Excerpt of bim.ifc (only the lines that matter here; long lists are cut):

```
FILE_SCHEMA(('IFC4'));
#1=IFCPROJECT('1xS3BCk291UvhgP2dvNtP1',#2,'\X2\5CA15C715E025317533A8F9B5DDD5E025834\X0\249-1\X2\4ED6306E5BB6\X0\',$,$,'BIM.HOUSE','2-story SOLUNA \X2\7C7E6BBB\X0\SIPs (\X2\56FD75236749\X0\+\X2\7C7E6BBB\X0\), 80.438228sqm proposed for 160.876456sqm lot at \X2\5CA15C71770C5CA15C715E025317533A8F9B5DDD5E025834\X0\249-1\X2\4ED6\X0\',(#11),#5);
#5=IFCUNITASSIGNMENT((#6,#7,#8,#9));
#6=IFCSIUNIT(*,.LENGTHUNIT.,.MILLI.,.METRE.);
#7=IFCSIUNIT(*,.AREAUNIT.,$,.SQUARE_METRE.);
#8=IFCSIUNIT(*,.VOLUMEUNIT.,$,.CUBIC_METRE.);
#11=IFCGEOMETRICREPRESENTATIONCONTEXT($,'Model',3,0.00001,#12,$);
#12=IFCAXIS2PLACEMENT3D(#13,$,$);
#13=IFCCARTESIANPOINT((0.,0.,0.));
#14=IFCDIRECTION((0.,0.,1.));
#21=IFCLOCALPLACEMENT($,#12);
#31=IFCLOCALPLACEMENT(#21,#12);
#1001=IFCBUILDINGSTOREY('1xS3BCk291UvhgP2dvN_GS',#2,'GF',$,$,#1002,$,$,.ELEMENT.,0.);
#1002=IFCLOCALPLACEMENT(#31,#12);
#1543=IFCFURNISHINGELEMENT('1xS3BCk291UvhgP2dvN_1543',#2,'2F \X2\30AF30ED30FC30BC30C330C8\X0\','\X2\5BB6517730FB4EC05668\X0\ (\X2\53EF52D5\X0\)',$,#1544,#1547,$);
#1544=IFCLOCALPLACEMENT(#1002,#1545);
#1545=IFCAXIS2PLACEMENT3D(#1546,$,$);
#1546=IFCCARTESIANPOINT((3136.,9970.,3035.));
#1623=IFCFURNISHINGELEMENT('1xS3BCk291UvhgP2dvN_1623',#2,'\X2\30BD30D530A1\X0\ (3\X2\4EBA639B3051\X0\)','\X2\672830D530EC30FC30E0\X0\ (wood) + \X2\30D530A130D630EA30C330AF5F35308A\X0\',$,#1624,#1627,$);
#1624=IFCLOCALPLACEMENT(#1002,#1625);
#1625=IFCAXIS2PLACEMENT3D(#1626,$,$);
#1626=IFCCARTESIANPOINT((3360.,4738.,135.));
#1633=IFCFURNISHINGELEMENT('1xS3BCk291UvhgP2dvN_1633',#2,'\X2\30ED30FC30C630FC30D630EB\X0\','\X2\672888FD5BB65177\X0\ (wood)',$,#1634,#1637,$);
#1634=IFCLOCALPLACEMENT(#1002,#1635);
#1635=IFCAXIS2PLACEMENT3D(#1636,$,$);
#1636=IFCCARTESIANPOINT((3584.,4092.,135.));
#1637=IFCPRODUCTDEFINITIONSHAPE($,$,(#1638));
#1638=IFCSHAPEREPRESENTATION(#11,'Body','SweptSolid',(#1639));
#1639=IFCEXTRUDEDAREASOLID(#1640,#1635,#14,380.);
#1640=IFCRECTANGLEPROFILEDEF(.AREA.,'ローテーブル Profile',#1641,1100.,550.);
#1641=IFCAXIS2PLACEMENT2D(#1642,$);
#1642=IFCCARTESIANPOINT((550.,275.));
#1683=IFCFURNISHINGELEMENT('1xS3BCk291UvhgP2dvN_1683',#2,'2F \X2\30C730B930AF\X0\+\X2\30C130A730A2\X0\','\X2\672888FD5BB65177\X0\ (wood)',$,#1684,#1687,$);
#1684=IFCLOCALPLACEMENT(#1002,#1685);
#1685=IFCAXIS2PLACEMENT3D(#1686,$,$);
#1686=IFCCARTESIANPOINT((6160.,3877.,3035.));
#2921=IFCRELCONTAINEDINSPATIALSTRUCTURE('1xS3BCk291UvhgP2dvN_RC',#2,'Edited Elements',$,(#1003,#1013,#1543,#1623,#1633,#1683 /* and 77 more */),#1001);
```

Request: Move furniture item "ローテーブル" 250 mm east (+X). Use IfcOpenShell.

```python
import ifcopenshell
import ifcopenshell.api.geometry
import ifcopenshell.util.placement

model = ifcopenshell.open("bim.ifc")

item = model.by_guid("1xS3BCk291UvhgP2dvN_1633")
matrix = ifcopenshell.util.placement.get_local_placement(item.ObjectPlacement)
matrix[0, 3] += 250.0
ifcopenshell.api.geometry.edit_object_placement(model, product=item, matrix=matrix, is_si=False)

print(ifcopenshell.util.placement.get_local_placement(item.ObjectPlacement).round(3) + 0.0)

model.write("bim_v2.ifc")
```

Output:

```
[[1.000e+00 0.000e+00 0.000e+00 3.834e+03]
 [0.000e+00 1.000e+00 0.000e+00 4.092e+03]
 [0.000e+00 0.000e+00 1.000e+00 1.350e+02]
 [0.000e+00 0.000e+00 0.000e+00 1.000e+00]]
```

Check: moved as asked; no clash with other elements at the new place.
